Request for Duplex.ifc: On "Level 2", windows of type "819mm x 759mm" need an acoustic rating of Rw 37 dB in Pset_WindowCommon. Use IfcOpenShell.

First a look at what the model holds.

```python
import ifcopenshell
import ifcopenshell.util.element

model = ifcopenshell.open("Duplex.ifc")
print(model.schema)
storey = next(s for s in model.by_type("IfcBuildingStorey") if s.Name == "Level 2")
windows = [e for e in ifcopenshell.util.element.get_decomposition(storey) if e.is_a("IfcWindow")]
seen = {}
for e in windows:
    element_type = ifcopenshell.util.element.get_type(e)
    key = (element_type.Name if element_type != e and element_type else None, ifcopenshell.util.element.get_pset(e, "Pset_WindowCommon", "AcousticRating"))
    seen[key] = seen.get(key, 0) + 1
for (name, value), count in sorted(seen.items(), key=str):
    print(count, "x", name, "|", value)
```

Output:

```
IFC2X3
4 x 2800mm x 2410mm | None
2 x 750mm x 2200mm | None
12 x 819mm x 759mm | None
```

```python
import ifcopenshell
import ifcopenshell.api.pset
import ifcopenshell.util.element

model = ifcopenshell.open("Duplex.ifc")

storey = next(s for s in model.by_type("IfcBuildingStorey") if s.Name == "Level 2")
windows = [e for e in ifcopenshell.util.element.get_decomposition(storey) if e.is_a("IfcWindow")]

count = 0
for e in windows:
    element_type = ifcopenshell.util.element.get_type(e)
    if element_type in (None, e) or element_type.Name != "819mm x 759mm":
        continue
    # add_pset returns the element's existing set when there is one.
    pset = ifcopenshell.api.pset.add_pset(model, product=e, name="Pset_WindowCommon")
    ifcopenshell.api.pset.edit_pset(model, pset=pset, properties={"AcousticRating": "Rw 37 dB"})
    count += 1

print(count, "windows updated")

model.write("Duplex_rev.ifc")
```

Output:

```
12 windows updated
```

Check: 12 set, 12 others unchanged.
